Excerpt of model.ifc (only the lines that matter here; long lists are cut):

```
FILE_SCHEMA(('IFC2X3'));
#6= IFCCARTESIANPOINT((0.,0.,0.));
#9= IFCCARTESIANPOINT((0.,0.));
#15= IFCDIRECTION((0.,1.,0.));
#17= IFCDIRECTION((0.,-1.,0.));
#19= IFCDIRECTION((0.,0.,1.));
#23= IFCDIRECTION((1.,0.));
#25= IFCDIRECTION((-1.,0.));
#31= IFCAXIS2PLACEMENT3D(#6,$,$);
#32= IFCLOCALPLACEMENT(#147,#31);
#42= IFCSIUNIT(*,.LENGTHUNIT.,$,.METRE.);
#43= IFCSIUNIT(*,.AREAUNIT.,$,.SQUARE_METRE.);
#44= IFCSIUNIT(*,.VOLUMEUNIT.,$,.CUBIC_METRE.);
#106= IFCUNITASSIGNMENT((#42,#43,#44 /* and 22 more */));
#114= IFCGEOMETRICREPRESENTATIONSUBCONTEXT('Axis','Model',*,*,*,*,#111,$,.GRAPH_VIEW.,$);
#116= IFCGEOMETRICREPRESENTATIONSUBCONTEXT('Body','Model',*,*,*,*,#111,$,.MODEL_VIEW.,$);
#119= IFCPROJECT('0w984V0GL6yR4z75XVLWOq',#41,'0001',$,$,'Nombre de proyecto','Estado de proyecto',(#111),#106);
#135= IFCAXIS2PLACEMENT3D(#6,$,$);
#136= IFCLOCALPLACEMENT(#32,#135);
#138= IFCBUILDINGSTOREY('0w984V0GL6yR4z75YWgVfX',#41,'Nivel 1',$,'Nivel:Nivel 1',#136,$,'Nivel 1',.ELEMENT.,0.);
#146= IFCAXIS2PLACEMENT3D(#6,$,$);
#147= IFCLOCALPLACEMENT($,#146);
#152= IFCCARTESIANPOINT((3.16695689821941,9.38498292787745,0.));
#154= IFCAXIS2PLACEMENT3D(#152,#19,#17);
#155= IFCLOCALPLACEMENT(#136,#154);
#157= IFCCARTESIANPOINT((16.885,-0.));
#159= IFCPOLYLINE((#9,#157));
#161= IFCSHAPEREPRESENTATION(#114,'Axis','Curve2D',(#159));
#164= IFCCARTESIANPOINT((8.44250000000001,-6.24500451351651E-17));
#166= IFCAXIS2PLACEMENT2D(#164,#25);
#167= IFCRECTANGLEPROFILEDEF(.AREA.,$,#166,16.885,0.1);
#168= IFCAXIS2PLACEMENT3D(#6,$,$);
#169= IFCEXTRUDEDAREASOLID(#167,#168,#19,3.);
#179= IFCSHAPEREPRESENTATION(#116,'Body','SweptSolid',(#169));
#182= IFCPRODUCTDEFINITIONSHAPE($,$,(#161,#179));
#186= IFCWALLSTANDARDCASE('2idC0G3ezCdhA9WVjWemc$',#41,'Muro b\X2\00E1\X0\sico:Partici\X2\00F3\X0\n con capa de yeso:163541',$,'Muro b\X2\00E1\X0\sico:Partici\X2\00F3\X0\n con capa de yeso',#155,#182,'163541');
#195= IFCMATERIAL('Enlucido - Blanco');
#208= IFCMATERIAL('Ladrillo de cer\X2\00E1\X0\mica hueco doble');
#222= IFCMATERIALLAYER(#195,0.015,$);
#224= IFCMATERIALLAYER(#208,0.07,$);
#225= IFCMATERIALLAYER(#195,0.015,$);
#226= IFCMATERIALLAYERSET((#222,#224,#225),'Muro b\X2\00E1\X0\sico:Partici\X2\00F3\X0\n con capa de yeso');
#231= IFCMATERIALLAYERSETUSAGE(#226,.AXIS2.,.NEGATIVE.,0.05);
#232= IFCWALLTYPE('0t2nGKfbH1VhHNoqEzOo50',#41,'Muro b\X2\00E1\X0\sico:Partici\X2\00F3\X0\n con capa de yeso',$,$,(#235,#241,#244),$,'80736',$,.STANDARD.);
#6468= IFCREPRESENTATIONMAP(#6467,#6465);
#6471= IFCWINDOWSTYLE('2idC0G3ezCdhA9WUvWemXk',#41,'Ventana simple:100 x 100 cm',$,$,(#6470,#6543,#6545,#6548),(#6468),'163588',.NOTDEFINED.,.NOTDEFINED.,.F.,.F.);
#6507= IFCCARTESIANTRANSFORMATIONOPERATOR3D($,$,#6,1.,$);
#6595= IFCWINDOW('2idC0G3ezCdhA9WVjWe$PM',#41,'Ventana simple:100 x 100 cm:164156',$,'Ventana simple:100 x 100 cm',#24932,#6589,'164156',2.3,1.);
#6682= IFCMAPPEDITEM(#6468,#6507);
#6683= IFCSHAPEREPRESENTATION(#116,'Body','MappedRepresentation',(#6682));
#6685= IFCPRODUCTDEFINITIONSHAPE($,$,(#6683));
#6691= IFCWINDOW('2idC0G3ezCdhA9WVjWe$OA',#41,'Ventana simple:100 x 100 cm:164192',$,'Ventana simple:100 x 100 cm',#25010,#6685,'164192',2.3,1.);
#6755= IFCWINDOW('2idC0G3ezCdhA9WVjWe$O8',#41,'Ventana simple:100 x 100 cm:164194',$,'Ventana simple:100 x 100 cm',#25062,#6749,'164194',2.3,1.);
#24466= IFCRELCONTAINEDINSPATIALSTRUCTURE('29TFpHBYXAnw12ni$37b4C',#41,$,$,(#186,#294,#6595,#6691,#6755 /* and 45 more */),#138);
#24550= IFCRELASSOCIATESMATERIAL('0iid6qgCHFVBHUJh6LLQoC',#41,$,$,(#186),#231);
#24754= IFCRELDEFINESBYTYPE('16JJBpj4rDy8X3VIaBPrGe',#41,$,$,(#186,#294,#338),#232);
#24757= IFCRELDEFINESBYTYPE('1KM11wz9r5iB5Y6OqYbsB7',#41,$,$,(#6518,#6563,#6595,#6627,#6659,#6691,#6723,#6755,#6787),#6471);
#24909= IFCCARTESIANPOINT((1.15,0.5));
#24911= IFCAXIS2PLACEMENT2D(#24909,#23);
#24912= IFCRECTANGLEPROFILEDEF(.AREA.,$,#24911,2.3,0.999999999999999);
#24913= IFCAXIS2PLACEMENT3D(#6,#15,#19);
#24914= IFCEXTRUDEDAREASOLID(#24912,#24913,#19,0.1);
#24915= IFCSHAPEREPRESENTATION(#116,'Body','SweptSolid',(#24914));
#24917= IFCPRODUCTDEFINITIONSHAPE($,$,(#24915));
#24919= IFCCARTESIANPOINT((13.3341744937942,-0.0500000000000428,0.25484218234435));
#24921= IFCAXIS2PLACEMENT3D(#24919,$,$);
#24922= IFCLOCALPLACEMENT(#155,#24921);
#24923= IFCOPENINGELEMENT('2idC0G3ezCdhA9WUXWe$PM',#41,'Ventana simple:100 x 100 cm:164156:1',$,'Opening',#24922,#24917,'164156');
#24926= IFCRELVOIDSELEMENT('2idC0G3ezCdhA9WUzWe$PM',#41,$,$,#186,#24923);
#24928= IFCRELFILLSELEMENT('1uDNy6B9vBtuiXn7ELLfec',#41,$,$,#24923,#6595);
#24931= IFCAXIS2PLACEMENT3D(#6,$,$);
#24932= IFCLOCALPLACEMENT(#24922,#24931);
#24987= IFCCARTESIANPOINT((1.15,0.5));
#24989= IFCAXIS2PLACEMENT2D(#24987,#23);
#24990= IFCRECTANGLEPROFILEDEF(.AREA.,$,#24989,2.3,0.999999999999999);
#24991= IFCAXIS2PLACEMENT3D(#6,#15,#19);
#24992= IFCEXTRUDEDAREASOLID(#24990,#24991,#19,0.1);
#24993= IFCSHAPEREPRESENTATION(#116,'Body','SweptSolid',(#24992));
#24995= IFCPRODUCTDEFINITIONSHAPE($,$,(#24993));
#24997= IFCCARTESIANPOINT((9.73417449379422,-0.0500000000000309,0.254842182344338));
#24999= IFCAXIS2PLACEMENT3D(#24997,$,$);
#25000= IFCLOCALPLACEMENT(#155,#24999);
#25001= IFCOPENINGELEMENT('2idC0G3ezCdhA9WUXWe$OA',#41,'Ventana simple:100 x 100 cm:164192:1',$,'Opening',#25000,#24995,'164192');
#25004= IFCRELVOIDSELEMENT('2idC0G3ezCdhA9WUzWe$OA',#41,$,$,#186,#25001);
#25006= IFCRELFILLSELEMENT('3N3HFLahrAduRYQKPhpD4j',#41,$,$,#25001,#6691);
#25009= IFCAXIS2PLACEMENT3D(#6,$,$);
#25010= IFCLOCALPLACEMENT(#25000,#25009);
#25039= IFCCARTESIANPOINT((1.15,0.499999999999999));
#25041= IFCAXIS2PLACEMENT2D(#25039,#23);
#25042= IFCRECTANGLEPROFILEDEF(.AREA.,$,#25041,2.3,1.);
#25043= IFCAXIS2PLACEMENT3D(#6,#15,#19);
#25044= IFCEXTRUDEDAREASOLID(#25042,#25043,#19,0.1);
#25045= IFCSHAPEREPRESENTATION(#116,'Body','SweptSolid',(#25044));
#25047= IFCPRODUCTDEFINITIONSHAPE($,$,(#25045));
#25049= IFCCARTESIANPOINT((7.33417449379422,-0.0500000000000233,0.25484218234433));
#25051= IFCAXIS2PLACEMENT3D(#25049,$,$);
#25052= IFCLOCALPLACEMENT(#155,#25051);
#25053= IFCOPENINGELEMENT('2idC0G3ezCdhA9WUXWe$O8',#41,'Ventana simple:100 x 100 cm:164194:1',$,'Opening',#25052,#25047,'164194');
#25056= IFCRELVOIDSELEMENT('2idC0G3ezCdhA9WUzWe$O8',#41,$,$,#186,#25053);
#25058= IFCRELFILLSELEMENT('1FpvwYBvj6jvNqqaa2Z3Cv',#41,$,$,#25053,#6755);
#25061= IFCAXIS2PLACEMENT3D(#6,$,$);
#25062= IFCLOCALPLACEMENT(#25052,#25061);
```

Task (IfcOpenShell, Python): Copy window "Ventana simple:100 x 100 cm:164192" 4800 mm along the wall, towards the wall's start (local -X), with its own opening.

```python
import ifcopenshell
import ifcopenshell.api.feature
import ifcopenshell.api.geometry
import ifcopenshell.api.root
import ifcopenshell.geom
import ifcopenshell.util.element
import ifcopenshell.util.placement
import ifcopenshell.util.shape
import ifcopenshell.util.unit

model = ifcopenshell.open("model.ifc")
unit_scale = ifcopenshell.util.unit.calculate_unit_scale(model)
settings = ifcopenshell.geom.settings()


def volume(element):
    """Net volume in cubic metres, openings subtracted."""
    shape = ifcopenshell.geom.create_shape(settings, element)
    return ifcopenshell.util.shape.get_volume(shape.geometry)


def reuse_history(source, copy):
    """copy_class also copies each property set's owner history, people and application; keep the originals."""
    for rel in copy.IsDefinedBy:
        if rel.is_a("IfcRelDefinesByProperties") and (history := rel.RelatingPropertyDefinition.OwnerHistory):
            rel.RelatingPropertyDefinition.OwnerHistory = source.OwnerHistory
            ifcopenshell.util.element.remove_deep2(model, history)


window = model.by_guid("2idC0G3ezCdhA9WVjWe$OA")
opening = window.FillsVoids[0].RelatingOpeningElement
wall = opening.VoidsElements[0].RelatingBuildingElement
before = volume(wall)
shift = ifcopenshell.util.placement.get_local_placement(wall.ObjectPlacement)[:3, 0] * -4.8 / unit_scale

# copy_class copies the void relationship, type, container and properties, but no geometry.
new_opening = ifcopenshell.api.root.copy_class(model, product=opening)
new_opening.Representation = ifcopenshell.util.element.copy_deep(
    model, opening.Representation, exclude=["IfcGeometricRepresentationContext", "IfcRepresentationMap"]
)
new_opening.Name = "Ventana simple:100 x 100 cm"
new_opening.Tag = None
new_window = ifcopenshell.api.root.copy_class(model, product=window)
new_window.Representation = ifcopenshell.util.element.copy_deep(
    model, window.Representation, exclude=["IfcGeometricRepresentationContext", "IfcRepresentationMap"]
)
new_window.Name = "Ventana simple:100 x 100 cm"
new_window.Tag = None
reuse_history(window, new_window)
fills = ifcopenshell.api.feature.add_filling(model, opening=new_opening, element=new_window)
fills.OwnerHistory = new_window.OwnerHistory  # required in IFC2X3

for old, new in ((opening, new_opening), (window, new_window)):
    matrix = ifcopenshell.util.placement.get_local_placement(old.ObjectPlacement)
    matrix[:3, 3] += shift
    ifcopenshell.api.geometry.edit_object_placement(model, product=new, matrix=matrix, is_si=False)

after = volume(wall)

print(f"wall volume {before:.3f} -> {after:.3f} m3")

model.write("model-out.ifc")
```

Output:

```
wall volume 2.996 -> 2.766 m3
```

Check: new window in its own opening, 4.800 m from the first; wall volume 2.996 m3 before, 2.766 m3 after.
